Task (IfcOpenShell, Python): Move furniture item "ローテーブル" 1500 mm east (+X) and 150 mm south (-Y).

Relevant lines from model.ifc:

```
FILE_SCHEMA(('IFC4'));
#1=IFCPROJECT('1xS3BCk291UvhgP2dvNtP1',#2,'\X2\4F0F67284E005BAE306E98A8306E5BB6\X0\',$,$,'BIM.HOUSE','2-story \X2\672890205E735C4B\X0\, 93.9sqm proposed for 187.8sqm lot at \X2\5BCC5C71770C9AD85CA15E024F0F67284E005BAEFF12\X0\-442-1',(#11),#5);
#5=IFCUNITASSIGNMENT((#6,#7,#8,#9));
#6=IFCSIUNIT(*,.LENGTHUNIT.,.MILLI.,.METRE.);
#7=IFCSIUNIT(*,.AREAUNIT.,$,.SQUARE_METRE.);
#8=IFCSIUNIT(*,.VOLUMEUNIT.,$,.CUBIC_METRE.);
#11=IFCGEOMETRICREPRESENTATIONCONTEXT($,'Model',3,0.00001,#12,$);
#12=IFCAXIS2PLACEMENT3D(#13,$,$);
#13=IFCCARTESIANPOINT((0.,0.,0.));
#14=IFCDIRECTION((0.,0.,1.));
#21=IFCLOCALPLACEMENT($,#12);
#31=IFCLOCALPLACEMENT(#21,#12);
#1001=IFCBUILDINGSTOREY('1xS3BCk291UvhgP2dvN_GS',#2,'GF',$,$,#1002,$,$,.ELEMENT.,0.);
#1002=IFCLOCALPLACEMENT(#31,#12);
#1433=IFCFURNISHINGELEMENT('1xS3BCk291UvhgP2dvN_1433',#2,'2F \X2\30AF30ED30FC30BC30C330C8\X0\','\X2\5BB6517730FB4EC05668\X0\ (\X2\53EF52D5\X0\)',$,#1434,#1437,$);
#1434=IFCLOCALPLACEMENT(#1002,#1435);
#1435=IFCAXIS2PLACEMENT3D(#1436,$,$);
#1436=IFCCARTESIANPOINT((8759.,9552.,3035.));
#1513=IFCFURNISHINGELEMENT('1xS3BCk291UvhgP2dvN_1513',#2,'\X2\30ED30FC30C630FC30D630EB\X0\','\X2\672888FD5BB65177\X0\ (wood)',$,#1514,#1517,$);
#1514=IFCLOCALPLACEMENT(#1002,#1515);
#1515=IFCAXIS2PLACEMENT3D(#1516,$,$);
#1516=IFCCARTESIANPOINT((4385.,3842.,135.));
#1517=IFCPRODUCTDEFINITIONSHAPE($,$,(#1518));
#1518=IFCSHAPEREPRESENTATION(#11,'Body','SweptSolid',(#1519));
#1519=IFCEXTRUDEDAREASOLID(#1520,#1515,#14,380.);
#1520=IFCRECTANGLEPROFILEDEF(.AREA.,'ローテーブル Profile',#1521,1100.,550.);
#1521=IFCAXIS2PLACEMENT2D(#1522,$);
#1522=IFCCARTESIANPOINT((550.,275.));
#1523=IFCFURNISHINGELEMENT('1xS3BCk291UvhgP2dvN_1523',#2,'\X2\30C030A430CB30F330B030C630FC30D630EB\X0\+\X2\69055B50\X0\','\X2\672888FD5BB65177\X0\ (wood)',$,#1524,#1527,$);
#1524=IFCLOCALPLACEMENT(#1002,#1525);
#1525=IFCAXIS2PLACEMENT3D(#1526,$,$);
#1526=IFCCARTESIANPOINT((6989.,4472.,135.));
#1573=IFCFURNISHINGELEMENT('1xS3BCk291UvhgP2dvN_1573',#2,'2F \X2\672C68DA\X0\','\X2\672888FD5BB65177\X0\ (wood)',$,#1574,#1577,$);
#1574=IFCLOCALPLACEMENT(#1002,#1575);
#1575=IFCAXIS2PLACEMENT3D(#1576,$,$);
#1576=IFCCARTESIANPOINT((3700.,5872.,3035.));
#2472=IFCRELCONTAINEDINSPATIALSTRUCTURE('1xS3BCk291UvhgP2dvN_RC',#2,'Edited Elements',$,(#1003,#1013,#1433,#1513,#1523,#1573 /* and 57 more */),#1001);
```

```python
import ifcopenshell
import ifcopenshell.api.geometry
import ifcopenshell.util.placement

model = ifcopenshell.open("model.ifc")

item = model.by_guid("1xS3BCk291UvhgP2dvN_1513")
matrix = ifcopenshell.util.placement.get_local_placement(item.ObjectPlacement)
matrix[0, 3] += 1500.0
matrix[1, 3] -= 150.0
ifcopenshell.api.geometry.edit_object_placement(model, product=item, matrix=matrix, is_si=False)

print(ifcopenshell.util.placement.get_local_placement(item.ObjectPlacement).round(3) + 0.0)

model.write("model_rev.ifc")
```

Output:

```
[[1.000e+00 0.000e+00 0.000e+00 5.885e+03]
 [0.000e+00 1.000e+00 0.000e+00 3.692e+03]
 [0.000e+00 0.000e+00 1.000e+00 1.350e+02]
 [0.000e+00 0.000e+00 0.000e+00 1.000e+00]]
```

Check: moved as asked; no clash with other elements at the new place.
